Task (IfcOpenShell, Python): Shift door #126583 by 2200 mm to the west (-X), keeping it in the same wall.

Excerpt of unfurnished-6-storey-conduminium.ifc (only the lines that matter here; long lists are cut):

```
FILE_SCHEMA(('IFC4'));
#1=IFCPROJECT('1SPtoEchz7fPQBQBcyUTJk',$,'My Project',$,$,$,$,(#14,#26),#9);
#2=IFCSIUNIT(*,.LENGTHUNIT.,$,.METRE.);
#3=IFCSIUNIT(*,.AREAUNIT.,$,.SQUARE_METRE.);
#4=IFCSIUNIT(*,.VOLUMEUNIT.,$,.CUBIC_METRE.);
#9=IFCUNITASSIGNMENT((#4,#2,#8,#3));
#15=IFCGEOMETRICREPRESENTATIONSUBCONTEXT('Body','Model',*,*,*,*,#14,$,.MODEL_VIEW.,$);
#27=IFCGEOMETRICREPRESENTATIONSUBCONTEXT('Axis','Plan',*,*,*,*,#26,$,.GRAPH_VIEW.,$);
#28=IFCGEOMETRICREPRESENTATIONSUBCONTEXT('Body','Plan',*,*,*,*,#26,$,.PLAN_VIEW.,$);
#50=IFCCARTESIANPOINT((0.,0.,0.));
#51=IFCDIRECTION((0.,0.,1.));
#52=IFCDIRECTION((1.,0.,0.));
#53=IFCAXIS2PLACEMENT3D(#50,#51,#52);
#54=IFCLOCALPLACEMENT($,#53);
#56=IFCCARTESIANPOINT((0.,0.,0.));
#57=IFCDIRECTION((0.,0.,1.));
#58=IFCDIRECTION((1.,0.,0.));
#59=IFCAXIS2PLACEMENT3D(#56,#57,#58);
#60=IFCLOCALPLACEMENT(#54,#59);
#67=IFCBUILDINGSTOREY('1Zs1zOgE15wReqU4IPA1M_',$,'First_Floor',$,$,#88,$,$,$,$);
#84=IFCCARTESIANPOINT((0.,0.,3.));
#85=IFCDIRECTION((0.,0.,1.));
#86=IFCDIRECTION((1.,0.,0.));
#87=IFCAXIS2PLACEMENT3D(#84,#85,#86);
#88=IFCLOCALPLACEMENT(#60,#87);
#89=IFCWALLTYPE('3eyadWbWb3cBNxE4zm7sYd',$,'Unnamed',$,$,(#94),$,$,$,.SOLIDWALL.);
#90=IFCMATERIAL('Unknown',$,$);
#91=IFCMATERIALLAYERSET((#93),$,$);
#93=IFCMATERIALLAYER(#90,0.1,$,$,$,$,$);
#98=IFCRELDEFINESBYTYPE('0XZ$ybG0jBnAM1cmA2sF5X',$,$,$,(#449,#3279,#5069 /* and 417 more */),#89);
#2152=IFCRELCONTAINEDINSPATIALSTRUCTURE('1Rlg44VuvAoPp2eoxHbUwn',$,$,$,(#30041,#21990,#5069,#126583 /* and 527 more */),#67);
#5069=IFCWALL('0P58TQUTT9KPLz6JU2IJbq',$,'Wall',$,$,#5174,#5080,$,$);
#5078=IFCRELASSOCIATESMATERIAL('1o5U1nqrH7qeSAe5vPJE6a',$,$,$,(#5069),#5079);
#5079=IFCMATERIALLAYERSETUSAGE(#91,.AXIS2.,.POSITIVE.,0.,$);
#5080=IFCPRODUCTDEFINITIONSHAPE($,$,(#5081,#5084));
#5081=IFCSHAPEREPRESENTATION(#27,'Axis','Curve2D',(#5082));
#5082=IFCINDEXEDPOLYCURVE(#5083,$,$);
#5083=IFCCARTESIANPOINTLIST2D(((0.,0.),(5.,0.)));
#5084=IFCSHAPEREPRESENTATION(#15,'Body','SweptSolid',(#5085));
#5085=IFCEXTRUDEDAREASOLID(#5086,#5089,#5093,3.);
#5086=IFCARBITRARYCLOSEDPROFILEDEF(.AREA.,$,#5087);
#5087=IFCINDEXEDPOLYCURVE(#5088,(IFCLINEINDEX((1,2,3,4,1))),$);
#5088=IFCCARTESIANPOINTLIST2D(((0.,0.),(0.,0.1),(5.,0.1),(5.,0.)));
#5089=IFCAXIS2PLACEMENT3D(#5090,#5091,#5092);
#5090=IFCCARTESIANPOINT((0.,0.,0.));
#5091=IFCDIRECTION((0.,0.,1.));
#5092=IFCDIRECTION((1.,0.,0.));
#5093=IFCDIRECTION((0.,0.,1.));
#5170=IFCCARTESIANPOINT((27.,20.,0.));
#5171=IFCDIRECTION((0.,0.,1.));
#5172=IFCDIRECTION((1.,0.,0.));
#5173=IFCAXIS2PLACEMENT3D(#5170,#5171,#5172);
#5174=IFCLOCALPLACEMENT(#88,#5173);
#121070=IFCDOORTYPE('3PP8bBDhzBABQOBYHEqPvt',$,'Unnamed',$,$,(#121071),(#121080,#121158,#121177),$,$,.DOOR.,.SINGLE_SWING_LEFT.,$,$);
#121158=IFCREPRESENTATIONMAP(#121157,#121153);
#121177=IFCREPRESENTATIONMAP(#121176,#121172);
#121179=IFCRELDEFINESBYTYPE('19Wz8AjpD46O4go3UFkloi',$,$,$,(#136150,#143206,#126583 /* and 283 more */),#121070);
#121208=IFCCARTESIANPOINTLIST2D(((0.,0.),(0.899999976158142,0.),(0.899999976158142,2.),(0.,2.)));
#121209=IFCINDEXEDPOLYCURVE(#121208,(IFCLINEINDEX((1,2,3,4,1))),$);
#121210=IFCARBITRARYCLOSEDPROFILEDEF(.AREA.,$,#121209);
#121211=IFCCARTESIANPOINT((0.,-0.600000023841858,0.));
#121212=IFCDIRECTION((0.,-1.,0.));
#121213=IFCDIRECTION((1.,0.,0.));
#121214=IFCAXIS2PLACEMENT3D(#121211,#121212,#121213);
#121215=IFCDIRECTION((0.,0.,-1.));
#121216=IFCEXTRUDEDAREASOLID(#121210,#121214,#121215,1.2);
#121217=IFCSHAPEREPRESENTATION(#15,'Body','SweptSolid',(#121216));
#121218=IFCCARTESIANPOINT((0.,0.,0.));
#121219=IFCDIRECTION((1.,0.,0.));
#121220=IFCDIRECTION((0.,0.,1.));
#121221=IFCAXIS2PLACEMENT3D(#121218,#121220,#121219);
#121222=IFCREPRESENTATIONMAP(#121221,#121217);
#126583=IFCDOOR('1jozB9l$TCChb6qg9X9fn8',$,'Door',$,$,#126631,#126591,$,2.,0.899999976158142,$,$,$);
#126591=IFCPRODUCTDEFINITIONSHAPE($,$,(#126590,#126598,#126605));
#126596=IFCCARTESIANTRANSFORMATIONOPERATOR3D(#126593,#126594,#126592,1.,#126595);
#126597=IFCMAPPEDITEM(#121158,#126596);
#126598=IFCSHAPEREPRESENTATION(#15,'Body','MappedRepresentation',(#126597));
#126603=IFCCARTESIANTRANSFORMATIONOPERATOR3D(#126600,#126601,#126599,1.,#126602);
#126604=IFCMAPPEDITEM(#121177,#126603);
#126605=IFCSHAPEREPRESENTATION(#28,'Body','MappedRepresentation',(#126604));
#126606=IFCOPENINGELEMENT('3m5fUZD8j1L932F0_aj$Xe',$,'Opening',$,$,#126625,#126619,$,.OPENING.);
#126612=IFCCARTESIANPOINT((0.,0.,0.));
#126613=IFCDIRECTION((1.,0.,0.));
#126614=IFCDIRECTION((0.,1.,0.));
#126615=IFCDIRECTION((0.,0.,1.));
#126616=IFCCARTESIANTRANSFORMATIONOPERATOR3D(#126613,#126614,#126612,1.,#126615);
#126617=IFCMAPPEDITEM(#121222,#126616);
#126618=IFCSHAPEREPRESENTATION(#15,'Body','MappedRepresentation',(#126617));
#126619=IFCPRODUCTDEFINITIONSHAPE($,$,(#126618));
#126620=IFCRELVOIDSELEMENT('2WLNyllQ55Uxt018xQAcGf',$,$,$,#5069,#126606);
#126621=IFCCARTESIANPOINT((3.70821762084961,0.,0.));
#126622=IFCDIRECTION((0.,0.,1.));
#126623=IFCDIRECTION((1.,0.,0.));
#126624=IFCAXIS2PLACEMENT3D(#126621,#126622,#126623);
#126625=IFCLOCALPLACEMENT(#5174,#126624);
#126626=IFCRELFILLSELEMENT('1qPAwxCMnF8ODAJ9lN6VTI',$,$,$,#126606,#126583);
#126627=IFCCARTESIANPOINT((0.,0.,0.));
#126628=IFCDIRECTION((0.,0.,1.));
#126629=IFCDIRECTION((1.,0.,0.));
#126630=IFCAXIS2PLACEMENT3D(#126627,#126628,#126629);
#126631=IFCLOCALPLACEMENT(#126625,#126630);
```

```python
import ifcopenshell
import ifcopenshell.api.geometry
import ifcopenshell.util.placement
import ifcopenshell.util.unit

model = ifcopenshell.open("unfurnished-6-storey-conduminium.ifc")
unit_scale = ifcopenshell.util.unit.calculate_unit_scale(model)

door = model.by_guid("1jozB9l$TCChb6qg9X9fn8")
opening = door.FillsVoids[0].RelatingOpeningElement
wall = opening.VoidsElements[0].RelatingBuildingElement

wall_matrix = ifcopenshell.util.placement.get_local_placement(wall.ObjectPlacement)
shift = wall_matrix[:3, 0] * -2.2 / unit_scale
before = ifcopenshell.util.placement.get_local_placement(door.ObjectPlacement)[:3, 3].copy()

# The door is placed relative to its opening, so it follows when the opening moves.
matrix = ifcopenshell.util.placement.get_local_placement(opening.ObjectPlacement)
matrix[:3, 3] += shift
ifcopenshell.api.geometry.edit_object_placement(
    model, product=opening, matrix=matrix, is_si=False, should_transform_children=True
)

after = ifcopenshell.util.placement.get_local_placement(door.ObjectPlacement)[:3, 3]
print("door moved by", (after - before).round(3) + 0.0)

model.write("unfurnished-6-storey-conduminium-out.ifc")
```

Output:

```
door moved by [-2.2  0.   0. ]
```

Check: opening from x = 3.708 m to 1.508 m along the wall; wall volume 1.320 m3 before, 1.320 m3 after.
